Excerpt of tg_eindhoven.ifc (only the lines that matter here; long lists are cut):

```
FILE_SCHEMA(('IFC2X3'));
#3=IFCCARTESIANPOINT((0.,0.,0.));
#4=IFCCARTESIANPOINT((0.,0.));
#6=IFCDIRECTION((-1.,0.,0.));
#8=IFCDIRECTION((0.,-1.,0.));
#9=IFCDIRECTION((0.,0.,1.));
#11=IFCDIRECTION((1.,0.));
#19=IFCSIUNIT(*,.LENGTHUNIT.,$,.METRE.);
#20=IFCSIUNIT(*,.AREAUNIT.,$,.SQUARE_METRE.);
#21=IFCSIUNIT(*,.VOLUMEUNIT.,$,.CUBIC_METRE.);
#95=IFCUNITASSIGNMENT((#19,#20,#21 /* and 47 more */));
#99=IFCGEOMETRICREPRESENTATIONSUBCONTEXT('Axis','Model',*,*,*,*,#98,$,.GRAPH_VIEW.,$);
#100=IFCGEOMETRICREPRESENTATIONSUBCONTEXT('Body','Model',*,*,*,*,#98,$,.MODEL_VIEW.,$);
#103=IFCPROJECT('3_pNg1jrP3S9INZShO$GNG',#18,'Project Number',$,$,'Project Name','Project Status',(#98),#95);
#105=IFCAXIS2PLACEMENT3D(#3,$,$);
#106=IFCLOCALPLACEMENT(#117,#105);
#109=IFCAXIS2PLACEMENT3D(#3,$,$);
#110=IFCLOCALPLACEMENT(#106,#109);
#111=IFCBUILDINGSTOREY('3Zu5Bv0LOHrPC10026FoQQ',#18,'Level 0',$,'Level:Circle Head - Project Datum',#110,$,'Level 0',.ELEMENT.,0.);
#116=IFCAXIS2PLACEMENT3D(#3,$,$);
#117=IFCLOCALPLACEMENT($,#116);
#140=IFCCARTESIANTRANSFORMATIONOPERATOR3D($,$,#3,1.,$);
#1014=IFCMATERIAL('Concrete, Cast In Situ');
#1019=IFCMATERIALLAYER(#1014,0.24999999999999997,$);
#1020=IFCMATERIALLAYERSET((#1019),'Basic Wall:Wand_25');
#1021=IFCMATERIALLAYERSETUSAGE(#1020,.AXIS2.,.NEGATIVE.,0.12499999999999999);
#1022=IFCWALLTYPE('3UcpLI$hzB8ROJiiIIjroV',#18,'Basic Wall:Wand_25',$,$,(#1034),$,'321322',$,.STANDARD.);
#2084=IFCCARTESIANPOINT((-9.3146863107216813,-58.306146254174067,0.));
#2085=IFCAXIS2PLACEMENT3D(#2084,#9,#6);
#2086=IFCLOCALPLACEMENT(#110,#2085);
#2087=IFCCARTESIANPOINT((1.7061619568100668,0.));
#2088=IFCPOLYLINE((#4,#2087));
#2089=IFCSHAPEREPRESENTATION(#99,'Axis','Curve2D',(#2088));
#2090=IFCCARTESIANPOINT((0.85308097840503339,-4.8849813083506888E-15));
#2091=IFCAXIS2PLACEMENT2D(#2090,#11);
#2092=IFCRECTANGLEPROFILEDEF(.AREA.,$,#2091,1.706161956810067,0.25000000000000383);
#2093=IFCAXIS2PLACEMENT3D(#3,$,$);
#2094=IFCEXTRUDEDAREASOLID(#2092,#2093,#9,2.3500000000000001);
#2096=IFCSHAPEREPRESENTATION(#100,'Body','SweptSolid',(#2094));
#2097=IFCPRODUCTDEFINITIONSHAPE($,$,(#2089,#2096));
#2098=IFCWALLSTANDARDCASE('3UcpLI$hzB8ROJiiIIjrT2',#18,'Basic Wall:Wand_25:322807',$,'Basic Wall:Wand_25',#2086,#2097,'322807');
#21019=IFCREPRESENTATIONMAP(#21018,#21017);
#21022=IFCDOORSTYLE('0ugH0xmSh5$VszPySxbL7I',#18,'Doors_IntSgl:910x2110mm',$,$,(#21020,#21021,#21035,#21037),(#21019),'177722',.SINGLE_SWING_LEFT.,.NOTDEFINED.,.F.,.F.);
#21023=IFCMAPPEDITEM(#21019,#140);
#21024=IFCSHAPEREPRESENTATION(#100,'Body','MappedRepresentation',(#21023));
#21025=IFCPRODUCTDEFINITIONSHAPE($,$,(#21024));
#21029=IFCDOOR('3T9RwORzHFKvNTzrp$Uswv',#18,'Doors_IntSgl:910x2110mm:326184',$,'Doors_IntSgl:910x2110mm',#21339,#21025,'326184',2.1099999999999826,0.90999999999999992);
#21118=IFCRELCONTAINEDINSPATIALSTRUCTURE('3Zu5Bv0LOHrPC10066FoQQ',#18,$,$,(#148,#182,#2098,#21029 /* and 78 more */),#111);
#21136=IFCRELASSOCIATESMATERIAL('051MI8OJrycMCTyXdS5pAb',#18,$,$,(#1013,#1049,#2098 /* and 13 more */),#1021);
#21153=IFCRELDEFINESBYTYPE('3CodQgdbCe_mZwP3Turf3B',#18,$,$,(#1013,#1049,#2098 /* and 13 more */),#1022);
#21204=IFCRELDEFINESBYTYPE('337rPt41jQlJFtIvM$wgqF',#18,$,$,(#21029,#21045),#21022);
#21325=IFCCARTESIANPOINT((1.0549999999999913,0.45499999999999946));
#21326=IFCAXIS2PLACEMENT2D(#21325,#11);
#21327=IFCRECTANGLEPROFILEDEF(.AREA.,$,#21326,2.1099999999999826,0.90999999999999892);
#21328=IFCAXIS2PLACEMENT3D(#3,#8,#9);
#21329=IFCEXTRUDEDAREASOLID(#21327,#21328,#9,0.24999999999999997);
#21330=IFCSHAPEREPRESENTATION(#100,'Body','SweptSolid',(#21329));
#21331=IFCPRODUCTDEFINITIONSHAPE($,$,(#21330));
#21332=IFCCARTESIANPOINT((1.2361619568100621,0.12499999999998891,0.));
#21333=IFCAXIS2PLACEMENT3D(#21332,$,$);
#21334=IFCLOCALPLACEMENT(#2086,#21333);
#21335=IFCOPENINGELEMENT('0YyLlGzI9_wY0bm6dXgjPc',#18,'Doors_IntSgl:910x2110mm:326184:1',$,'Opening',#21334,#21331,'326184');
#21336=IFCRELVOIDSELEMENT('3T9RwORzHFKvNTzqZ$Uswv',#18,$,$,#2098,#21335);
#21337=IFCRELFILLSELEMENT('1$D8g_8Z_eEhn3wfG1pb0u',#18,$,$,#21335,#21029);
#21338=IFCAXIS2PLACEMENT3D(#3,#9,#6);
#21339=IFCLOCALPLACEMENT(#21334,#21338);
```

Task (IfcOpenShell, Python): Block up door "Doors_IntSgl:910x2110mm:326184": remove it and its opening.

```python
import ifcopenshell
import ifcopenshell.api.feature
import ifcopenshell.api.root
import ifcopenshell.geom
import ifcopenshell.util.shape

model = ifcopenshell.open("tg_eindhoven.ifc")
settings = ifcopenshell.geom.settings()


def volume(element):
    """Net volume in cubic metres, openings subtracted."""
    shape = ifcopenshell.geom.create_shape(settings, element)
    return ifcopenshell.util.shape.get_volume(shape.geometry)


door = model.by_guid("3T9RwORzHFKvNTzrp$Uswv")
opening = door.FillsVoids[0].RelatingOpeningElement
wall = opening.VoidsElements[0].RelatingBuildingElement
before = volume(wall)

ifcopenshell.api.root.remove_product(model, product=door)
ifcopenshell.api.feature.remove_feature(model, feature=opening)

after = volume(wall)

print(f"wall volume {before:.3f} -> {after:.3f} m3")

model.write("tg_eindhoven_rev.ifc")
```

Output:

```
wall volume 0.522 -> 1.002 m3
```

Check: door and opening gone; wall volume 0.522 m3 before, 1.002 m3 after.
